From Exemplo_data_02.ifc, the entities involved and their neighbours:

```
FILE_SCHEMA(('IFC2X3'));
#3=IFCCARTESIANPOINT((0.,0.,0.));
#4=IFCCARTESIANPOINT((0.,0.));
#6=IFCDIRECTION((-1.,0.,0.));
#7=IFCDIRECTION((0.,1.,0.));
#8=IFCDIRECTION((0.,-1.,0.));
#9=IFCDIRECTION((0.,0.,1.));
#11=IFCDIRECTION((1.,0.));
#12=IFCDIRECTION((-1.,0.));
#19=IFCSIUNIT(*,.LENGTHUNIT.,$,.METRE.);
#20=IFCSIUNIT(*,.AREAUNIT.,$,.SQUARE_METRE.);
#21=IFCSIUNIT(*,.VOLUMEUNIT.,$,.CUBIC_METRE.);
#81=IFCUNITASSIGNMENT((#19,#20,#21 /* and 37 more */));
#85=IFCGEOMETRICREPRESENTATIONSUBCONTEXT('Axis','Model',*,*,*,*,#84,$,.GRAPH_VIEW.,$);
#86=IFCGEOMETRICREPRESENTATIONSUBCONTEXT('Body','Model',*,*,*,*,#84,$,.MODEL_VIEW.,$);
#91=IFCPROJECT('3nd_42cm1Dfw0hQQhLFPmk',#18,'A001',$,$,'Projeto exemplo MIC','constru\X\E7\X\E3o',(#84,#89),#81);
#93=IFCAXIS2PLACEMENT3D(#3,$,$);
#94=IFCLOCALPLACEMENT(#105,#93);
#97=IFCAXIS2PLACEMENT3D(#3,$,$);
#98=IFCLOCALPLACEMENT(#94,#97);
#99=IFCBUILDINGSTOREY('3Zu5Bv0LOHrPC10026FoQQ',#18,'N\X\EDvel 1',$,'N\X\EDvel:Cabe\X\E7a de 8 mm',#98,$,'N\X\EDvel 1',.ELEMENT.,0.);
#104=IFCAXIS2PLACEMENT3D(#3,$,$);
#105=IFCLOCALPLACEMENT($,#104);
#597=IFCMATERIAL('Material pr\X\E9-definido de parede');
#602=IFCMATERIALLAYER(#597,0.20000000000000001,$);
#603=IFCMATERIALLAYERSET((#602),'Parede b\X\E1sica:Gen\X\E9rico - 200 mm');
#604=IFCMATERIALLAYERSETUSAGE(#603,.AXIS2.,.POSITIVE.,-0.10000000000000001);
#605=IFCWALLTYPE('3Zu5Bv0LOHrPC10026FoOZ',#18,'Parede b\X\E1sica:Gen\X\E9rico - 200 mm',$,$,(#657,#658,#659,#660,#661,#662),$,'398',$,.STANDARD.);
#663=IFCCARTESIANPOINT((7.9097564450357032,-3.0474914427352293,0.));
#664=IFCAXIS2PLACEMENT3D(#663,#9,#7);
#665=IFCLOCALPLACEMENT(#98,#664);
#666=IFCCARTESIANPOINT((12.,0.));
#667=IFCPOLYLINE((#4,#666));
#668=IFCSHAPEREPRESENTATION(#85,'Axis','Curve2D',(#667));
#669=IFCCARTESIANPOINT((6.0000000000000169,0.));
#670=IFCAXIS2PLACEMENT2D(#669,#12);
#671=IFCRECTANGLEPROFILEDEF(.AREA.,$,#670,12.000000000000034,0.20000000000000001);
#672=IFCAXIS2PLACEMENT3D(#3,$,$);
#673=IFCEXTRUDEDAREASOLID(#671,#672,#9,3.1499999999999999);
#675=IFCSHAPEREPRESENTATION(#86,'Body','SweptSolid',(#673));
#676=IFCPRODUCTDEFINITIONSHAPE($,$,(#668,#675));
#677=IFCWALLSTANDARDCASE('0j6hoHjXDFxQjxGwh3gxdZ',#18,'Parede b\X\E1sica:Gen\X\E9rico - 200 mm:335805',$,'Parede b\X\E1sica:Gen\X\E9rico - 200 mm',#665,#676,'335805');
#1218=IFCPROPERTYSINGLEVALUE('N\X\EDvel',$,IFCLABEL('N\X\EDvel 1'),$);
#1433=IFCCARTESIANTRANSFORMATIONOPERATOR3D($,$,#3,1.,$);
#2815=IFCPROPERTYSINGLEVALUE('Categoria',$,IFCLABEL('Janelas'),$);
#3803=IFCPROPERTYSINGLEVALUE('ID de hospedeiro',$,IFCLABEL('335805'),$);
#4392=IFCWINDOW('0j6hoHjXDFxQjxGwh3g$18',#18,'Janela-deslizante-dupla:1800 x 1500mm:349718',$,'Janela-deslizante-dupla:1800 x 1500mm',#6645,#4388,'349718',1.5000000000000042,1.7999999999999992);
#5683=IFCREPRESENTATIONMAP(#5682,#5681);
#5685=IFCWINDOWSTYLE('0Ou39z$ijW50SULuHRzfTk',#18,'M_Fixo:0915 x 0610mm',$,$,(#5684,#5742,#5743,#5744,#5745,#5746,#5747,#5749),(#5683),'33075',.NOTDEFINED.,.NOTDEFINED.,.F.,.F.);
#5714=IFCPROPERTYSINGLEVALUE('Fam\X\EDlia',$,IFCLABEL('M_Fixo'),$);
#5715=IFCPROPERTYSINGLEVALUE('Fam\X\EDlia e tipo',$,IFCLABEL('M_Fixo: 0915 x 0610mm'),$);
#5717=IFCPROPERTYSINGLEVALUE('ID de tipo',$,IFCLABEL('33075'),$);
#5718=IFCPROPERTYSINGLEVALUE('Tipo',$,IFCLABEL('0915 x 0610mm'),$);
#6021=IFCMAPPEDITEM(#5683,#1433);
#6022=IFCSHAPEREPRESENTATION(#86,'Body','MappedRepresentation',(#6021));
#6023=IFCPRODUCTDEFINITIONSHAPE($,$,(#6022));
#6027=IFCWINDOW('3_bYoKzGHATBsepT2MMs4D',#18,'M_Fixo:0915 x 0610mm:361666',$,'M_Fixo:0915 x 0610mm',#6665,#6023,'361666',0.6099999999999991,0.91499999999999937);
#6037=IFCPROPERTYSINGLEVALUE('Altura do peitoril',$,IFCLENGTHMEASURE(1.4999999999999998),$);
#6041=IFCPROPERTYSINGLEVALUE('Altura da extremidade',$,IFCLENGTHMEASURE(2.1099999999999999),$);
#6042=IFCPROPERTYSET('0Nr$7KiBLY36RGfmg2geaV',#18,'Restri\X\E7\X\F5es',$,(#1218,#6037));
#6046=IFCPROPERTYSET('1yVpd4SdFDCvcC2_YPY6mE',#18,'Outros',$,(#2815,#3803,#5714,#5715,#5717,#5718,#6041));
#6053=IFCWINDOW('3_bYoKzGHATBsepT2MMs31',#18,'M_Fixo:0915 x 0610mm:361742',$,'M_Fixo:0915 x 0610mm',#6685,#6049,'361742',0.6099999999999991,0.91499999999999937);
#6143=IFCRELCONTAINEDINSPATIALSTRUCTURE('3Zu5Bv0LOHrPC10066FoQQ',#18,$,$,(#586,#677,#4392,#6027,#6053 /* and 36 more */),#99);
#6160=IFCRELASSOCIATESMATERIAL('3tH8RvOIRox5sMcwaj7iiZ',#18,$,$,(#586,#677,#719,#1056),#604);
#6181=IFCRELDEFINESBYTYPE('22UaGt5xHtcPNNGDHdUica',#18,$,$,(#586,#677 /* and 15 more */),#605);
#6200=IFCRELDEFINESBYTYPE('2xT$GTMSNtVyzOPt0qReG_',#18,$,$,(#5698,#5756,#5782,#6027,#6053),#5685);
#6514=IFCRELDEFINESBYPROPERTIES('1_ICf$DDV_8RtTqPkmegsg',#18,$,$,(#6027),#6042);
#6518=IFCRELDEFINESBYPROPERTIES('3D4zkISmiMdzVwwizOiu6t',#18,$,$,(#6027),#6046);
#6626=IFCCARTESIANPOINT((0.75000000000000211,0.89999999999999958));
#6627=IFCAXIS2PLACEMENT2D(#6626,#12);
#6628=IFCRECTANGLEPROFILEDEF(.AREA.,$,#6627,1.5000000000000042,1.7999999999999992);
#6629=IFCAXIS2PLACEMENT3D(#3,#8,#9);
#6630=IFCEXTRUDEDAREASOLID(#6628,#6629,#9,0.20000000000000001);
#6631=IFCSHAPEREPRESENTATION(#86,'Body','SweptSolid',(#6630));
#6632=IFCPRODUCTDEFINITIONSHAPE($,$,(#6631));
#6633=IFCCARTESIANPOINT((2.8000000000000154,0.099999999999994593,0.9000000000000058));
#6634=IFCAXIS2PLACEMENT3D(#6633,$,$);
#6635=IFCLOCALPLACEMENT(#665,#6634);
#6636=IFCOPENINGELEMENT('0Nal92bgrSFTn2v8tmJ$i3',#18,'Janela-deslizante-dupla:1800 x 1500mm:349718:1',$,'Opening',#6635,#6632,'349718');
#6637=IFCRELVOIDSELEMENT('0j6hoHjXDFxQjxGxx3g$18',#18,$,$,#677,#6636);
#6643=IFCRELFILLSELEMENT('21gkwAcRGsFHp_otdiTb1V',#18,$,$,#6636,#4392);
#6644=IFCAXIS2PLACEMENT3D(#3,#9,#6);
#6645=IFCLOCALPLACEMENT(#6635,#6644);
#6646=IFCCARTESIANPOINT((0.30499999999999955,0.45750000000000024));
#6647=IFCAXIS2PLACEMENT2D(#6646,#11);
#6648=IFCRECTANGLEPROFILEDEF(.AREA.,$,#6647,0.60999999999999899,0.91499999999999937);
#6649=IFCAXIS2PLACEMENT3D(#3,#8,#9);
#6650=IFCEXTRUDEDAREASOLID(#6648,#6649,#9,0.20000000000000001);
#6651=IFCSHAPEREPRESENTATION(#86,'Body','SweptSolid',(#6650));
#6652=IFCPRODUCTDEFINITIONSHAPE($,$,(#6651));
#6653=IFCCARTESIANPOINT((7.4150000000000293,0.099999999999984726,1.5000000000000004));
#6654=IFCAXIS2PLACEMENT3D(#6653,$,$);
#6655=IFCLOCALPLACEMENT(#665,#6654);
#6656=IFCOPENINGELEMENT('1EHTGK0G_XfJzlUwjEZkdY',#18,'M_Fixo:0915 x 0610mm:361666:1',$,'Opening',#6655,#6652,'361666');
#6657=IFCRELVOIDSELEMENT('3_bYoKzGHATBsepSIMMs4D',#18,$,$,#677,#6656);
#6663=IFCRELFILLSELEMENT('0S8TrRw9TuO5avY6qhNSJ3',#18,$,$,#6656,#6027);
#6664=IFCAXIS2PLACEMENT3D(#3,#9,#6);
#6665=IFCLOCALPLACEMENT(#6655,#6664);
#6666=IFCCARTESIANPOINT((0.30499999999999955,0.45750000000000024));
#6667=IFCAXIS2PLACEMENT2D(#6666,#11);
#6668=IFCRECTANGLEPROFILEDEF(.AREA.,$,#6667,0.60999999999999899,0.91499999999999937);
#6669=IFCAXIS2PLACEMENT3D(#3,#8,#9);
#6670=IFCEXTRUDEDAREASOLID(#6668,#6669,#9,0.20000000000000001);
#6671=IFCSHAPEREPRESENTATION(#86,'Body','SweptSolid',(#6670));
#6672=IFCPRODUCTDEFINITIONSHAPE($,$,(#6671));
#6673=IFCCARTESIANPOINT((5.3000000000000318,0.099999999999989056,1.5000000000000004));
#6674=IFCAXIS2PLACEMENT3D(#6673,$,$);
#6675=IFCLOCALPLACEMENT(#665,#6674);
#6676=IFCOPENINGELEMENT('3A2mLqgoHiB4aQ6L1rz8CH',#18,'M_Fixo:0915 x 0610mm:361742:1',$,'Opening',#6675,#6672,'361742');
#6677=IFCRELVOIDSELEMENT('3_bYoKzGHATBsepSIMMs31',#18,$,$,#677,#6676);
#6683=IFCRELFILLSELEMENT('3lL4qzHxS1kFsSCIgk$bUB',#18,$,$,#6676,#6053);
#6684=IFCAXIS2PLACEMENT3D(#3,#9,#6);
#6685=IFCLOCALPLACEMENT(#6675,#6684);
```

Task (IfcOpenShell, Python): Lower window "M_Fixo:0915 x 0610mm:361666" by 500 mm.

```python
import numpy as np
import ifcopenshell
import ifcopenshell.api.geometry
import ifcopenshell.api.pset
import ifcopenshell.util.element
import ifcopenshell.util.placement
import ifcopenshell.util.unit

model = ifcopenshell.open("Exemplo_data_02.ifc")
unit_scale = ifcopenshell.util.unit.calculate_unit_scale(model)

window = model.by_guid("3_bYoKzGHATBsepT2MMs4D")
opening = window.FillsVoids[0].RelatingOpeningElement
dz = -0.5 / unit_scale

shift = np.array([0.0, 0.0, dz])
# The window is placed relative to its opening, so it follows when the opening moves.
matrix = ifcopenshell.util.placement.get_local_placement(opening.ObjectPlacement)
matrix[:3, 3] += shift
ifcopenshell.api.geometry.edit_object_placement(
    model, product=opening, matrix=matrix, is_si=False, should_transform_children=True
)

# Keep the stored heights in step.
pset = model.by_id(ifcopenshell.util.element.get_pset(window, "Restrições", should_inherit=False)["id"])
ifcopenshell.api.pset.edit_pset(model, pset=pset, properties={
    "Altura do peitoril": model.create_entity("IfcLengthMeasure", ifcopenshell.util.element.get_pset(window, "Restrições", "Altura do peitoril") + dz),
})
pset = model.by_id(ifcopenshell.util.element.get_pset(window, "Outros", should_inherit=False)["id"])
ifcopenshell.api.pset.edit_pset(model, pset=pset, properties={
    "Altura da extremidade": model.create_entity("IfcLengthMeasure", ifcopenshell.util.element.get_pset(window, "Outros", "Altura da extremidade") + dz),
})

print(f"moved by {dz * unit_scale:+.3f} m")

model.write("Exemplo_data_02_edited.ifc")
```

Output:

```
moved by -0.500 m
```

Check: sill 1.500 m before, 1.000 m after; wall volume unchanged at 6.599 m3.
